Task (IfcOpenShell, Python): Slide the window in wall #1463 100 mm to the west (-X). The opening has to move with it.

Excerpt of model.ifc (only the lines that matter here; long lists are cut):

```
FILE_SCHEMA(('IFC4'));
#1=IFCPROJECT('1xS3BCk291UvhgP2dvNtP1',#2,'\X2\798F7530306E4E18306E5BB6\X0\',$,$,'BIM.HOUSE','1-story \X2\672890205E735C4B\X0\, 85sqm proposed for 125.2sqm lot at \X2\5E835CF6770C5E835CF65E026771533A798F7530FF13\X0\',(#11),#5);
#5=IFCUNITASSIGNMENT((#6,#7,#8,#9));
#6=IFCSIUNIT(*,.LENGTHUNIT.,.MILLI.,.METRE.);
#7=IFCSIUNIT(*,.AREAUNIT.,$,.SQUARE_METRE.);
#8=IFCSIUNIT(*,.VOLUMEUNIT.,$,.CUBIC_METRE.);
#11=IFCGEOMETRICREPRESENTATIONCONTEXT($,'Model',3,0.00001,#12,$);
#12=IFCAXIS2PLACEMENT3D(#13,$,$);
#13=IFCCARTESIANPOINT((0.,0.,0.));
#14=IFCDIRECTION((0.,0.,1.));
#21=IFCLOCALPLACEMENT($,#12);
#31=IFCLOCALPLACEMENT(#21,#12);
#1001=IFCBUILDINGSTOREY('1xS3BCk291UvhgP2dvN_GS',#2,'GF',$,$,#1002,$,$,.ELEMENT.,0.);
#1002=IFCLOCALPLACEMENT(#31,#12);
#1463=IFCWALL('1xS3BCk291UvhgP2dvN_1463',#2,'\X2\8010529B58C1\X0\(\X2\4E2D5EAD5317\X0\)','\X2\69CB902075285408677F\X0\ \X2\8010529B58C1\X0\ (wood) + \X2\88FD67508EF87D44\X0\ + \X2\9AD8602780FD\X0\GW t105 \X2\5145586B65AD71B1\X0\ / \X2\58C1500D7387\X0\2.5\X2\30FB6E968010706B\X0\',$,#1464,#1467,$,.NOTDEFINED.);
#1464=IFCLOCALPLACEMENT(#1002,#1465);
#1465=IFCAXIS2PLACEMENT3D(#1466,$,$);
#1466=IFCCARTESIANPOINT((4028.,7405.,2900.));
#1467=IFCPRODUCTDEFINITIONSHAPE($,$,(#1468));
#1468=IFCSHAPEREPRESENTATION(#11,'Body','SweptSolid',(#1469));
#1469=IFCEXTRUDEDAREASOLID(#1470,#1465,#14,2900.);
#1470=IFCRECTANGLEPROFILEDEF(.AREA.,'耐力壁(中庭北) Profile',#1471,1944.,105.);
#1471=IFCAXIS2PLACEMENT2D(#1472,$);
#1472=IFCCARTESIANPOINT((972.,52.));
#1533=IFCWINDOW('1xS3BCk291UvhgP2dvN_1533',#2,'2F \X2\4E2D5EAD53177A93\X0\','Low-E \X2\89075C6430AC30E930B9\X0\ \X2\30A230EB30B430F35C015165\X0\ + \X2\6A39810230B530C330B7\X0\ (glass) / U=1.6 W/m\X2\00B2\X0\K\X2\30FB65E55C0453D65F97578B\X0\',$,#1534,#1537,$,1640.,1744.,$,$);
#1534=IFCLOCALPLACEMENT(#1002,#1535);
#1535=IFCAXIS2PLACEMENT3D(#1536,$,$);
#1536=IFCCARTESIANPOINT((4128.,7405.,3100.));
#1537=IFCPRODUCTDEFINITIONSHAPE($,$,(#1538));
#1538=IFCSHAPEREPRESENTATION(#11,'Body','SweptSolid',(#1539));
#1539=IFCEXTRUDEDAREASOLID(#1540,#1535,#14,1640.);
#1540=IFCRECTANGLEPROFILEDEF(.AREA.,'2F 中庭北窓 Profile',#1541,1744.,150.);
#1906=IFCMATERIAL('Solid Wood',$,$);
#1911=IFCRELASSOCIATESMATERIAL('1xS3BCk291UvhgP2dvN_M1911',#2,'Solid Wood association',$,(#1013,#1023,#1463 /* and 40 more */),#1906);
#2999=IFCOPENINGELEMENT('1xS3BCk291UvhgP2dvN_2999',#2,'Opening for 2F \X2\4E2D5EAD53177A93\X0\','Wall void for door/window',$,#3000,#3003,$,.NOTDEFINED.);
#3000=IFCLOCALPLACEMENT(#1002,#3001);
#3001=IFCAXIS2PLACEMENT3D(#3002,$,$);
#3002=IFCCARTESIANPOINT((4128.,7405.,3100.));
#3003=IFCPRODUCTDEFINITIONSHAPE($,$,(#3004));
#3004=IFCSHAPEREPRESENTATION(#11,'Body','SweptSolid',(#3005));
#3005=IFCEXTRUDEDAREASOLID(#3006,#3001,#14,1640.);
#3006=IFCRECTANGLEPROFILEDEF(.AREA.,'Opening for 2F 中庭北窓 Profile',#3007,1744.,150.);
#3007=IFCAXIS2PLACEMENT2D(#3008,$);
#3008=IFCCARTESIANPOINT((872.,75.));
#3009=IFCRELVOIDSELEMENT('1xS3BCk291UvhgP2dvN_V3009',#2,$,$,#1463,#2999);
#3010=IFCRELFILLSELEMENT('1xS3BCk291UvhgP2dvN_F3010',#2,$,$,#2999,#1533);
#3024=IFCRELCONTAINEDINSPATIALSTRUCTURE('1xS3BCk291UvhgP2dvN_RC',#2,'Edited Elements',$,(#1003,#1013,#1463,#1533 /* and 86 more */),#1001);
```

```python
import ifcopenshell
import ifcopenshell.api.geometry
import ifcopenshell.util.placement

model = ifcopenshell.open("model.ifc")

window = model.by_guid("1xS3BCk291UvhgP2dvN_1533")
opening = window.FillsVoids[0].RelatingOpeningElement
wall = opening.VoidsElements[0].RelatingBuildingElement

wall_matrix = ifcopenshell.util.placement.get_local_placement(wall.ObjectPlacement)
shift = wall_matrix[:3, 0] * -100.0
before = ifcopenshell.util.placement.get_local_placement(window.ObjectPlacement)[:3, 3].copy()

# The window is not placed relative to its opening, so move both.
for product in (opening, window):
    matrix = ifcopenshell.util.placement.get_local_placement(product.ObjectPlacement)
    matrix[:3, 3] += shift
    ifcopenshell.api.geometry.edit_object_placement(model, product=product, matrix=matrix, is_si=False)

after = ifcopenshell.util.placement.get_local_placement(window.ObjectPlacement)[:3, 3]
print("window moved by", (after - before).round(3) + 0.0)

model.write("model_edited.ifc")
```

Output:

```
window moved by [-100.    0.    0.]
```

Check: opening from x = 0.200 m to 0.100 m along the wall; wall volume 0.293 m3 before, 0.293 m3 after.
